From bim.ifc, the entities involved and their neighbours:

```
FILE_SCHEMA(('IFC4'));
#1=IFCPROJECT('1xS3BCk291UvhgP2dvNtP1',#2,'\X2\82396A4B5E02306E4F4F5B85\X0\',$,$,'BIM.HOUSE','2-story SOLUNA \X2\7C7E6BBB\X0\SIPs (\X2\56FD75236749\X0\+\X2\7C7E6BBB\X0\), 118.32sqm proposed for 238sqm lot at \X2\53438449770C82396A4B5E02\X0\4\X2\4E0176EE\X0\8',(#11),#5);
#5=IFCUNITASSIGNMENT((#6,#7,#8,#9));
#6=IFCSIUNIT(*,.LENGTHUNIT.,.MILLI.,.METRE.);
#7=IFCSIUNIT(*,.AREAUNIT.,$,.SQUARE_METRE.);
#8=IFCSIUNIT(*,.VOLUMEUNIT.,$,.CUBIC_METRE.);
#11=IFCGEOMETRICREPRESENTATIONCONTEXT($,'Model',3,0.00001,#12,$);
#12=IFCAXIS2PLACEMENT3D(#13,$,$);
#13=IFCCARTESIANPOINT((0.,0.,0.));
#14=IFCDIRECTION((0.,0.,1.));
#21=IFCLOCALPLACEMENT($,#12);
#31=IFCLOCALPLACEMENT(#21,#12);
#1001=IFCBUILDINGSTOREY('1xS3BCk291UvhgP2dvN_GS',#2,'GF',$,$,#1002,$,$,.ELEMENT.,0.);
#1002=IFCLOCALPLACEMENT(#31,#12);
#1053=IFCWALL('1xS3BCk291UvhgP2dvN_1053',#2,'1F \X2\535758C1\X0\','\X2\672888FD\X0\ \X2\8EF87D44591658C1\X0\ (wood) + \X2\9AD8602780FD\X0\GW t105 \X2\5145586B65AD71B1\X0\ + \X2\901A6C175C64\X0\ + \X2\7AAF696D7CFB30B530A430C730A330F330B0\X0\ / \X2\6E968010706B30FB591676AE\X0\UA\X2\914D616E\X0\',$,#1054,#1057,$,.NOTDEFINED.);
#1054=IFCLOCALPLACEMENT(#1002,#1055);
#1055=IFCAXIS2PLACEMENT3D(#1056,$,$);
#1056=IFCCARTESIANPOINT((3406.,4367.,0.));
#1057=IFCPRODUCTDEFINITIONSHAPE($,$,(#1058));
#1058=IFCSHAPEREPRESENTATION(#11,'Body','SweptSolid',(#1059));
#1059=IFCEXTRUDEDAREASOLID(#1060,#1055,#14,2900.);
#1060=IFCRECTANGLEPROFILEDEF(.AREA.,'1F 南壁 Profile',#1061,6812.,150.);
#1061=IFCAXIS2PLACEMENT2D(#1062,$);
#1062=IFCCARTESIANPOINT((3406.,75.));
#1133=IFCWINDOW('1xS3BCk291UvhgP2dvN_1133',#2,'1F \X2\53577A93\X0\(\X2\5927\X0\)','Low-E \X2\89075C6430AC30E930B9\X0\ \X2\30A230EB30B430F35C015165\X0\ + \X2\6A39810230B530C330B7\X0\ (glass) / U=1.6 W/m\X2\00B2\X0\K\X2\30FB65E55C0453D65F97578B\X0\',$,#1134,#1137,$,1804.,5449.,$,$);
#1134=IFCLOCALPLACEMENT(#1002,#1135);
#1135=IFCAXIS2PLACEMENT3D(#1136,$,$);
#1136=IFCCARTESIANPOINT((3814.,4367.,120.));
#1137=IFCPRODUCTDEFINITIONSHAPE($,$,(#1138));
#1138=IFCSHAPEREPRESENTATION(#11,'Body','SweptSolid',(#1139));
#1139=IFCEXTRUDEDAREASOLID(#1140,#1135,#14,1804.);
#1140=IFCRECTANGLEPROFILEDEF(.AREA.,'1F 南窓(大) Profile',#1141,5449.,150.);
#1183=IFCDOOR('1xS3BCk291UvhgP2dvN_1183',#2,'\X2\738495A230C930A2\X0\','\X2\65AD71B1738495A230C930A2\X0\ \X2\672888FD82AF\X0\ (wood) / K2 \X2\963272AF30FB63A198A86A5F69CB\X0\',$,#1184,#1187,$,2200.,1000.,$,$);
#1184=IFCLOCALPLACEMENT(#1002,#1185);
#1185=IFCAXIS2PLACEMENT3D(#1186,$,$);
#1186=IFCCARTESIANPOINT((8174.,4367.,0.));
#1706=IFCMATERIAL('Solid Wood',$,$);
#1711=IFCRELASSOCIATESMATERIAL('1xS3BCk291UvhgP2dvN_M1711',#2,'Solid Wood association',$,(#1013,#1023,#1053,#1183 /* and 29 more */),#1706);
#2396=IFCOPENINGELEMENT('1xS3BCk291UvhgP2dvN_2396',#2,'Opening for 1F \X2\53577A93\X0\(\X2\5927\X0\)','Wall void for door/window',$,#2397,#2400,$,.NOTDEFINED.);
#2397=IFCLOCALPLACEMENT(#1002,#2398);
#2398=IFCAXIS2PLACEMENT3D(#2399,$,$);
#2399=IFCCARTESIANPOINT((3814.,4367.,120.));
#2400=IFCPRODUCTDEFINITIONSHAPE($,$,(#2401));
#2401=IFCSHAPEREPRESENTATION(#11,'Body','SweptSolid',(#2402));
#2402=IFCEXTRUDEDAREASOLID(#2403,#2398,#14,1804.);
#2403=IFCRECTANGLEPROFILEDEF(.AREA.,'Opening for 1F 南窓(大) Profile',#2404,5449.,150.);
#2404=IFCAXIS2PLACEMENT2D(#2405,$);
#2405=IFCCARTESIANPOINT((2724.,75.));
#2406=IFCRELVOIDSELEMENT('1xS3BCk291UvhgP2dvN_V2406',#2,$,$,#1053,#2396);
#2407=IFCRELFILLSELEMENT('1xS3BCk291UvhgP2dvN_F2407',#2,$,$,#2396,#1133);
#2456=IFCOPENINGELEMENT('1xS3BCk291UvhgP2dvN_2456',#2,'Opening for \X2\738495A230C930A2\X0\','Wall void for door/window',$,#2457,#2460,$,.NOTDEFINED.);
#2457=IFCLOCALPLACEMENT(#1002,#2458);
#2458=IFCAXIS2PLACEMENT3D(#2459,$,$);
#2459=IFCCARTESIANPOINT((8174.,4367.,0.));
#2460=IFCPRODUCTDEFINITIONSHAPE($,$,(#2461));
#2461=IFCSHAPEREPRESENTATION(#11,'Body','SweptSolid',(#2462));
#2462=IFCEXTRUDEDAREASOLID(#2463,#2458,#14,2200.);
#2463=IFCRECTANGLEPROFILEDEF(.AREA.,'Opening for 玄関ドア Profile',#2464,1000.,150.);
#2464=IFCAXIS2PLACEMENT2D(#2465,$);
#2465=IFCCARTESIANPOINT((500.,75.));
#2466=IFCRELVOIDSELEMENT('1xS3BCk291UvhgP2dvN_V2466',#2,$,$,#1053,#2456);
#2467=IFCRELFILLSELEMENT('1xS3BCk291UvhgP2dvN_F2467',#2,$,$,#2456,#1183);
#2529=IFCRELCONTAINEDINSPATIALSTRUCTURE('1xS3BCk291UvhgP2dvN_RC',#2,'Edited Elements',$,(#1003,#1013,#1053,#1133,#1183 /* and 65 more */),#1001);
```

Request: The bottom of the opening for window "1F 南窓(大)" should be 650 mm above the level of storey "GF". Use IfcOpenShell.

```python
import numpy as np
import ifcopenshell
import ifcopenshell.api.geometry
import ifcopenshell.geom
import ifcopenshell.util.element
import ifcopenshell.util.placement
import ifcopenshell.util.shape
import ifcopenshell.util.unit

model = ifcopenshell.open("bim.ifc")
unit_scale = ifcopenshell.util.unit.calculate_unit_scale(model)

window = model.by_guid("1xS3BCk291UvhgP2dvN_1133")
opening = window.FillsVoids[0].RelatingOpeningElement
storey = ifcopenshell.util.element.get_container(window, ifc_class="IfcBuildingStorey")
level = ifcopenshell.util.placement.get_local_placement(storey.ObjectPlacement)[2, 3]

# The opening's origin need not be at the sill, so measure its lowest point.
shape = ifcopenshell.geom.create_shape(ifcopenshell.geom.settings(), opening)
bottom = ifcopenshell.util.shape.get_shape_bottom_elevation(shape, shape.geometry) / unit_scale
dz = level + 0.65 / unit_scale - bottom

shift = np.array([0.0, 0.0, dz])
# The window is not placed relative to its opening, so move both.
for product in (opening, window):
    matrix = ifcopenshell.util.placement.get_local_placement(product.ObjectPlacement)
    matrix[:3, 3] += shift
    ifcopenshell.api.geometry.edit_object_placement(model, product=product, matrix=matrix, is_si=False)

print(f"moved by {dz * unit_scale:+.3f} m")

model.write("bim_rev.ifc")
```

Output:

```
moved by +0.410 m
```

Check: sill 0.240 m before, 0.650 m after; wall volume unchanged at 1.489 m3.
